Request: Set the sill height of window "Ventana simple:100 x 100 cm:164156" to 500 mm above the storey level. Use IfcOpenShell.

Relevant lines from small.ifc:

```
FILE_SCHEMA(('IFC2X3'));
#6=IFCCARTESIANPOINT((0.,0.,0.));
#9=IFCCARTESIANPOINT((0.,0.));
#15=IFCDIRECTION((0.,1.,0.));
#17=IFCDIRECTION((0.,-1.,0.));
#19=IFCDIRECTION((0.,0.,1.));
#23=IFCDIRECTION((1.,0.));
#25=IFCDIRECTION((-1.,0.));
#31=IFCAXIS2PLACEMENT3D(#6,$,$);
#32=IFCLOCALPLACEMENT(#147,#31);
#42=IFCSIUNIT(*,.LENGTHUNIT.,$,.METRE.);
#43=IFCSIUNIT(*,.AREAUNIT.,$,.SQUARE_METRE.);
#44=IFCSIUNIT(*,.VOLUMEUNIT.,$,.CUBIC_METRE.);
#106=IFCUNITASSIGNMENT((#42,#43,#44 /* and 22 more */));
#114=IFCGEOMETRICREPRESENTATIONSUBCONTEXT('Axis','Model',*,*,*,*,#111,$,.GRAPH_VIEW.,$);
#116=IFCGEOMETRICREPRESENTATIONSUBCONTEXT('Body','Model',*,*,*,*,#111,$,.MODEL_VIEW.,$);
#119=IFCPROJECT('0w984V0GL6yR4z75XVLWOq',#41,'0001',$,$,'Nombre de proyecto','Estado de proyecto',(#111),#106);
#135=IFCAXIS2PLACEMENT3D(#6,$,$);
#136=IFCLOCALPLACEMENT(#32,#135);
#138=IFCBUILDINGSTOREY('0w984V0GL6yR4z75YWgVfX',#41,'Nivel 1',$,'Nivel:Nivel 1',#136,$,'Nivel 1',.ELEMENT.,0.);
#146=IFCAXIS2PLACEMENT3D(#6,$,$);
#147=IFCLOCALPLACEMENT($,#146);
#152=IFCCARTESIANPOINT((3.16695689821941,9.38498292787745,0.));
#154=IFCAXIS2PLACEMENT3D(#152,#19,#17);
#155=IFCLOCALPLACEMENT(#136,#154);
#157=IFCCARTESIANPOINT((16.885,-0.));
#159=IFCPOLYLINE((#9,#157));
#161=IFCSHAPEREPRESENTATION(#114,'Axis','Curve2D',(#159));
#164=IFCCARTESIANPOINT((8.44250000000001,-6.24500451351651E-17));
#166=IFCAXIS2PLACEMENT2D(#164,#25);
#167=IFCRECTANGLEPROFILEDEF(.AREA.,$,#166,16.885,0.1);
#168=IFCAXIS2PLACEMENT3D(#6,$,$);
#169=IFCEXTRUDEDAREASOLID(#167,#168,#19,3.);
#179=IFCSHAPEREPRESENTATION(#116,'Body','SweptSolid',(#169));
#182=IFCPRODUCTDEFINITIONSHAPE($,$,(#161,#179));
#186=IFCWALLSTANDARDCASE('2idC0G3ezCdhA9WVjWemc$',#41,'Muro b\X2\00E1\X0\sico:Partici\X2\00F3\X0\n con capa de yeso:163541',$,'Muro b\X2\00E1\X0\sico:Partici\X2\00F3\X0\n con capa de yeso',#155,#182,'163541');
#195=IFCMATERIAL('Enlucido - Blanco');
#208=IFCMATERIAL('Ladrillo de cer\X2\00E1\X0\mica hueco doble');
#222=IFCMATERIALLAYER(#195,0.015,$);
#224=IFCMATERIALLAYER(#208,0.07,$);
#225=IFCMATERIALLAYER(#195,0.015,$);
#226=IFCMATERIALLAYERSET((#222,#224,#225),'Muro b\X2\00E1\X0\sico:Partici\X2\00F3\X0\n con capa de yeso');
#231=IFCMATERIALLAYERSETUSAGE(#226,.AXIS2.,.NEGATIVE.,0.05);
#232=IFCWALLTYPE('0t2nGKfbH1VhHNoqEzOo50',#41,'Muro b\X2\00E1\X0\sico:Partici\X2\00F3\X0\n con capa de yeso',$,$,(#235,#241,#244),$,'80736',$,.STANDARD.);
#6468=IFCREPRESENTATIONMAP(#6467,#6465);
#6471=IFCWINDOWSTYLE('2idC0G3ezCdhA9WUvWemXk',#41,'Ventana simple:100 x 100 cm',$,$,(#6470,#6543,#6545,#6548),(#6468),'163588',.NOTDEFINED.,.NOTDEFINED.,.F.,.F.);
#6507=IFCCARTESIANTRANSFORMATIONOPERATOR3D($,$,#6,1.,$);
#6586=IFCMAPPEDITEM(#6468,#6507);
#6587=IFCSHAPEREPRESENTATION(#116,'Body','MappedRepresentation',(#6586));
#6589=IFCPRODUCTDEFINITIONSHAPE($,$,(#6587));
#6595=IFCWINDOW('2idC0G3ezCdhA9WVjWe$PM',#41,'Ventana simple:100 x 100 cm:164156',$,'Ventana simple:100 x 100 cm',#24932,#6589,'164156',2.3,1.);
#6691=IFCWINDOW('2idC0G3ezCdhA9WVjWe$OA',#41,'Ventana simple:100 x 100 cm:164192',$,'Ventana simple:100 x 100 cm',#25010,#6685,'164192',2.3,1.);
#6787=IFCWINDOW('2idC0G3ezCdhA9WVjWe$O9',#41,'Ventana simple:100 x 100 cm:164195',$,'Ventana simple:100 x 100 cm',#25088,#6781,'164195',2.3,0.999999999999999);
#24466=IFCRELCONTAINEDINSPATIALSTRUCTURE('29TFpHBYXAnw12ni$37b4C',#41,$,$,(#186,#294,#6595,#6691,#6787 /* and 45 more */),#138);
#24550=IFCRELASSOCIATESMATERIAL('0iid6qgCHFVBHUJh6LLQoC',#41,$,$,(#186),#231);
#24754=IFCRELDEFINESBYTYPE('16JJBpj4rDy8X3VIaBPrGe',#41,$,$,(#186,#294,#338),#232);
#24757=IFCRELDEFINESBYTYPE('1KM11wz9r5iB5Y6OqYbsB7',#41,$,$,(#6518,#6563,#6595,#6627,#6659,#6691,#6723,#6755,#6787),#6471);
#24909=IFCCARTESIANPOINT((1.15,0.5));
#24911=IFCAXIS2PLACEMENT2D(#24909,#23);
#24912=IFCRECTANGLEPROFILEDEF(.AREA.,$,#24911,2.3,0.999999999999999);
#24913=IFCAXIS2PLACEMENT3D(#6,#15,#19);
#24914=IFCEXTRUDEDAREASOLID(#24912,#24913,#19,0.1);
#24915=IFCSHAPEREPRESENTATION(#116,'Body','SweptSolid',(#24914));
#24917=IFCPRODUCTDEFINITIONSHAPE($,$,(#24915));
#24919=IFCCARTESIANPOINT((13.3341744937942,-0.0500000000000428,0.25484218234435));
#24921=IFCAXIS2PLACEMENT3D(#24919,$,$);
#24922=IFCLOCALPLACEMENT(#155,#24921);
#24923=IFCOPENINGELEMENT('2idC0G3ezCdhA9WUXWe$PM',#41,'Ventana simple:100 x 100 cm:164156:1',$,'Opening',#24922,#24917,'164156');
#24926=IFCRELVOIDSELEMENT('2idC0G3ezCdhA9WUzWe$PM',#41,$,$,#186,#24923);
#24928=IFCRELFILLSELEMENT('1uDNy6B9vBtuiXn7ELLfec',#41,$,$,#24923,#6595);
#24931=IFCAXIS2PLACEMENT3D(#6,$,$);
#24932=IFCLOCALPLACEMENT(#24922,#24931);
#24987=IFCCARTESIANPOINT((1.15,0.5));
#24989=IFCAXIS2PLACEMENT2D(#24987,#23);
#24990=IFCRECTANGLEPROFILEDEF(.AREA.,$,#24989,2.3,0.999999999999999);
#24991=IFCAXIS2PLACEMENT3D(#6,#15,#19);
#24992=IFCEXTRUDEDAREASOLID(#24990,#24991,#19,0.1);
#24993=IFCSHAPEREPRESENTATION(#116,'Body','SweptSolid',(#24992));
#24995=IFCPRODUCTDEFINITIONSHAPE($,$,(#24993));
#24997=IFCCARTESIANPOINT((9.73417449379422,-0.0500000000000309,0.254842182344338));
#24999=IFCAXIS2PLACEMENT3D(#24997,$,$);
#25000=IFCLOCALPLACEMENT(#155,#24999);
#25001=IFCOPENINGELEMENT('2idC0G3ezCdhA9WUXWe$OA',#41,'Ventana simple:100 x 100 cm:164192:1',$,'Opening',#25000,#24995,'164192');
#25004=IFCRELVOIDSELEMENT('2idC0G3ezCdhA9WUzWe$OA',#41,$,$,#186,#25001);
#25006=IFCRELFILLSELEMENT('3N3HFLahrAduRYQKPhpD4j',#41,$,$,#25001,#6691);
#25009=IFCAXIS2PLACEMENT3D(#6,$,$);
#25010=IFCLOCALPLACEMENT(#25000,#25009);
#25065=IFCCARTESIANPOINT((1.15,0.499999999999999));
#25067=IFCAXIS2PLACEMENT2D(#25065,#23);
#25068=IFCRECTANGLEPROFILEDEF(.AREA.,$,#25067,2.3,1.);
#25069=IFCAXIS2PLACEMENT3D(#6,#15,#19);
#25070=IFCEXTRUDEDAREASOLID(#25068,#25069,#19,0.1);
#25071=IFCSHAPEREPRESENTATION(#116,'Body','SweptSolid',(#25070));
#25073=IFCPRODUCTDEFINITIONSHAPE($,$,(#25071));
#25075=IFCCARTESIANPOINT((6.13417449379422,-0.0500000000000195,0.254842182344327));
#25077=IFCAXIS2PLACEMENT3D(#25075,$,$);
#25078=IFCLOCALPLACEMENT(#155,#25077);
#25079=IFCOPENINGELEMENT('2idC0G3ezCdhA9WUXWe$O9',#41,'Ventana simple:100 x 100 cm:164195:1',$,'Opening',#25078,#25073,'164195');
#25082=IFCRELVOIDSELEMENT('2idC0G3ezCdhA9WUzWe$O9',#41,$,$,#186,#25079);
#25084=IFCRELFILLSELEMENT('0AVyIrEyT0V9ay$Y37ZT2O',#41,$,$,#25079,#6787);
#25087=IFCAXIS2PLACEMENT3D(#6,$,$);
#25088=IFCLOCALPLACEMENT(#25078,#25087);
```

```python
import numpy as np
import ifcopenshell
import ifcopenshell.api.geometry
import ifcopenshell.geom
import ifcopenshell.util.element
import ifcopenshell.util.placement
import ifcopenshell.util.shape
import ifcopenshell.util.unit

model = ifcopenshell.open("small.ifc")
unit_scale = ifcopenshell.util.unit.calculate_unit_scale(model)

window = model.by_guid("2idC0G3ezCdhA9WVjWe$PM")
opening = window.FillsVoids[0].RelatingOpeningElement
storey = ifcopenshell.util.element.get_container(window, ifc_class="IfcBuildingStorey")
level = ifcopenshell.util.placement.get_local_placement(storey.ObjectPlacement)[2, 3]

# The opening's origin need not be at the sill, so measure its lowest point.
shape = ifcopenshell.geom.create_shape(ifcopenshell.geom.settings(), opening)
bottom = ifcopenshell.util.shape.get_shape_bottom_elevation(shape, shape.geometry) / unit_scale
dz = level + 0.5 / unit_scale - bottom

shift = np.array([0.0, 0.0, dz])
# The window is placed relative to its opening, so it follows when the opening moves.
matrix = ifcopenshell.util.placement.get_local_placement(opening.ObjectPlacement)
matrix[:3, 3] += shift
ifcopenshell.api.geometry.edit_object_placement(
    model, product=opening, matrix=matrix, is_si=False, should_transform_children=True
)

print(f"moved by {dz * unit_scale:+.3f} m")

model.write("small_rev.ifc")
```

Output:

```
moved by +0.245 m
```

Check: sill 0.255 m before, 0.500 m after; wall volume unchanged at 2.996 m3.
